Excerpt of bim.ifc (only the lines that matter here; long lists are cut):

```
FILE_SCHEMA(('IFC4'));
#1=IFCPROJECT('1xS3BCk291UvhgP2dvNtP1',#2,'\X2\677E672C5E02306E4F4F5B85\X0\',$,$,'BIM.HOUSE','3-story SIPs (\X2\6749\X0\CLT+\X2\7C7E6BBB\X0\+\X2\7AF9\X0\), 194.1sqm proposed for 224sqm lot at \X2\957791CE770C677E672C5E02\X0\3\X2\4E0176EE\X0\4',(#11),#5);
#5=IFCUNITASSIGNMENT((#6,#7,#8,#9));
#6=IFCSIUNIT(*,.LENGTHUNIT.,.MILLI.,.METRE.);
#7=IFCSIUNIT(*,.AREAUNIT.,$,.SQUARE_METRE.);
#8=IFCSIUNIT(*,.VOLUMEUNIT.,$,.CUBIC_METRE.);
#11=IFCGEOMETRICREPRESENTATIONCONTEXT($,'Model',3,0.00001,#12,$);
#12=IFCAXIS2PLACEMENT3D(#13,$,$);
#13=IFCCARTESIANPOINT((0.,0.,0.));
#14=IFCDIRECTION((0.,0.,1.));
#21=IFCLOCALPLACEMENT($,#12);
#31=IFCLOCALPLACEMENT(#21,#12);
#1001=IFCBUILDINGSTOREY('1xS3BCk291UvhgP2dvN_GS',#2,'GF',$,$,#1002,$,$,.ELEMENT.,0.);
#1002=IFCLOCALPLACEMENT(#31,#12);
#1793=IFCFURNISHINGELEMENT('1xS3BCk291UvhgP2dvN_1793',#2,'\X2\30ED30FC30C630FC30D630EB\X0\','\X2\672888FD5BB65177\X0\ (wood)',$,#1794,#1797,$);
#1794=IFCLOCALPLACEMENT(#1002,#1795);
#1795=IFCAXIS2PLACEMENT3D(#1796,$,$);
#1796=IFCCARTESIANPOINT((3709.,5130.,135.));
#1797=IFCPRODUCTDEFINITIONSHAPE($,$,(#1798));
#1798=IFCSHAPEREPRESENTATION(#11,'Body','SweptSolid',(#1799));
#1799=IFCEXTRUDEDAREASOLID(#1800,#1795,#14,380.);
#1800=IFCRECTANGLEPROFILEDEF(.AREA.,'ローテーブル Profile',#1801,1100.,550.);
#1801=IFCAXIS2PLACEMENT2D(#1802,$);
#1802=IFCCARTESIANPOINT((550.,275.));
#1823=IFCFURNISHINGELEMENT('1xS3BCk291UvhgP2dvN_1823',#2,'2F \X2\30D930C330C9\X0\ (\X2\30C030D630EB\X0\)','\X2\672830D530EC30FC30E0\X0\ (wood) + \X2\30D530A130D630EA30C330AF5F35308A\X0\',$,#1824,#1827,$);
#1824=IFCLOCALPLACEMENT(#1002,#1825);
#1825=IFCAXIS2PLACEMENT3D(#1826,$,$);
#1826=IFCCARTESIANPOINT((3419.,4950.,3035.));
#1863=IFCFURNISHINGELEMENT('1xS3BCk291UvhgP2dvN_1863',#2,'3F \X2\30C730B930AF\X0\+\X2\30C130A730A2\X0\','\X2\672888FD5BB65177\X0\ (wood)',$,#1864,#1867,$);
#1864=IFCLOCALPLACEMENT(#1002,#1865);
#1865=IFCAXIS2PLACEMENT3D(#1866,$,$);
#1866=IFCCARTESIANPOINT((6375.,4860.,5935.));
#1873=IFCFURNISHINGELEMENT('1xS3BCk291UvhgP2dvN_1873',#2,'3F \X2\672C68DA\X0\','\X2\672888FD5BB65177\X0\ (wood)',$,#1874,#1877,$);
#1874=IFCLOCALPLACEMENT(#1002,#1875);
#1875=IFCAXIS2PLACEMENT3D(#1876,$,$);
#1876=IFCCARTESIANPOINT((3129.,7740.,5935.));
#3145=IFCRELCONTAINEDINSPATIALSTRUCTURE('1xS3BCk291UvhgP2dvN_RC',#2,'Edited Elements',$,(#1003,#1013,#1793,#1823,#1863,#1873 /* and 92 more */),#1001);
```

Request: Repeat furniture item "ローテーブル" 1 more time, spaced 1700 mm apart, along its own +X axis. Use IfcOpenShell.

```python
import ifcopenshell
import ifcopenshell.api.geometry
import ifcopenshell.api.root
import ifcopenshell.util.element
import ifcopenshell.util.placement

model = ifcopenshell.open("bim.ifc")


def reuse_history(source, copy):
    """copy_class also copies each property set's owner history, people and application; keep the originals."""
    for rel in copy.IsDefinedBy:
        if rel.is_a("IfcRelDefinesByProperties") and (history := rel.RelatingPropertyDefinition.OwnerHistory):
            rel.RelatingPropertyDefinition.OwnerHistory = source.OwnerHistory
            ifcopenshell.util.element.remove_deep2(model, history)


source = model.by_guid("1xS3BCk291UvhgP2dvN_1793")
base = ifcopenshell.util.placement.get_local_placement(source.ObjectPlacement)
step = base[:3, 0] * 1700.0

for i in range(1, 2):
    copy = ifcopenshell.api.root.copy_class(model, product=source)
    copy.Representation = ifcopenshell.util.element.copy_deep(
        model, source.Representation, exclude=["IfcGeometricRepresentationContext", "IfcRepresentationMap"]
    )
    reuse_history(source, copy)
    matrix = base.copy()
    matrix[:3, 3] += i * step
    print("added at", matrix[:3, 3].round(3) + 0.0)
    ifcopenshell.api.geometry.edit_object_placement(model, product=copy, matrix=matrix, is_si=False)

model.write("bim_v2.ifc")
```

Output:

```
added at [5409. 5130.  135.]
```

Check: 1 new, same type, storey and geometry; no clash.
